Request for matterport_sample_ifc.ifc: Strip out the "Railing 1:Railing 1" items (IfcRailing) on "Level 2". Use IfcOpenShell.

First a look at what the model holds.

```python
import ifcopenshell
import ifcopenshell.util.element

model = ifcopenshell.open("matterport_sample_ifc.ifc")
print(model.schema)
storey = next(s for s in model.by_type("IfcBuildingStorey") if s.Name == "Level 2")
railings = [e for e in ifcopenshell.util.element.get_decomposition(storey) if e.is_a("IfcRailing")]
seen = {}
for e in railings:
    element_type = ifcopenshell.util.element.get_type(e)
    name = element_type.Name if element_type not in (None, e) else None
    seen[name] = seen.get(name, 0) + 1
for name, count in sorted(seen.items(), key=str):
    print(count, "x", name)
```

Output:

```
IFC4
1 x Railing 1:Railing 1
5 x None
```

```python
import ifcopenshell
import ifcopenshell.api.root
import ifcopenshell.util.element

model = ifcopenshell.open("matterport_sample_ifc.ifc")

storey = next(s for s in model.by_type("IfcBuildingStorey") if s.Name == "Level 2")
railings = [e for e in ifcopenshell.util.element.get_decomposition(storey) if e.is_a("IfcRailing")]
targets = [e for e in railings if (t := ifcopenshell.util.element.get_type(e)) not in (None, e) and t.Name == "Railing 1:Railing 1"]

for e in targets:
    ifcopenshell.api.root.remove_product(model, product=e)
print(len(targets), "removed")

model.write("matterport_sample_ifc_updated.ifc")
```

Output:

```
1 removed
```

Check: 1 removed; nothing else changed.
